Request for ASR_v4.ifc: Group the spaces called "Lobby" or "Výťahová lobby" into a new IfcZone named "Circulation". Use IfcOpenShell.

First a look at what the model holds.

```python
import ifcopenshell

model = ifcopenshell.open("ASR_v4.ifc")
print(model.schema)
seen = {}
for space in model.by_type("IfcSpace"):
    seen[space.LongName] = seen.get(space.LongName, 0) + 1
for name, count in sorted(seen.items(), key=str):
    print(count, "x", name)
print("zones:", [z.Name for z in model.by_type("IfcZone")][:20])
```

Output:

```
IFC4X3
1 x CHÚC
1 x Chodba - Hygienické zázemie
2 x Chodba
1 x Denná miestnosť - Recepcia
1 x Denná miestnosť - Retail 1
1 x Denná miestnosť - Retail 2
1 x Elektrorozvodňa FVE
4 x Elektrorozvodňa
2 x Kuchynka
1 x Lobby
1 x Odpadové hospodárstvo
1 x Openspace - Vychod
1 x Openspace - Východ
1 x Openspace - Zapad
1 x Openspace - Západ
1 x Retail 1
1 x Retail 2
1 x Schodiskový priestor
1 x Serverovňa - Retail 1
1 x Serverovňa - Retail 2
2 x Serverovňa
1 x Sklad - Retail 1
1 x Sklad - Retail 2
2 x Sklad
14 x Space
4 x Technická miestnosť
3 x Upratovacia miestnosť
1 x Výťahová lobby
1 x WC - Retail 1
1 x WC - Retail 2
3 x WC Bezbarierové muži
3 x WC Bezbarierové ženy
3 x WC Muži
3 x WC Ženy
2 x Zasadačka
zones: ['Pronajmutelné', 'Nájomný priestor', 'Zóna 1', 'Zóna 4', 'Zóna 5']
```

```python
import ifcopenshell
import ifcopenshell.api.group
import ifcopenshell.api.root

model = ifcopenshell.open("ASR_v4.ifc")

names = {"Lobby", "Výťahová lobby"}
spaces = [s for s in model.by_type("IfcSpace") if s.LongName in names]

zone = ifcopenshell.api.root.create_entity(model, ifc_class="IfcZone", name="Circulation")
ifcopenshell.api.group.assign_group(model, products=spaces, group=zone)
print(len(spaces), "spaces in", zone.Name)

model.write("ASR_v4_v2.ifc")
```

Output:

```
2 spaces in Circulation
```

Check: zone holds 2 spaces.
